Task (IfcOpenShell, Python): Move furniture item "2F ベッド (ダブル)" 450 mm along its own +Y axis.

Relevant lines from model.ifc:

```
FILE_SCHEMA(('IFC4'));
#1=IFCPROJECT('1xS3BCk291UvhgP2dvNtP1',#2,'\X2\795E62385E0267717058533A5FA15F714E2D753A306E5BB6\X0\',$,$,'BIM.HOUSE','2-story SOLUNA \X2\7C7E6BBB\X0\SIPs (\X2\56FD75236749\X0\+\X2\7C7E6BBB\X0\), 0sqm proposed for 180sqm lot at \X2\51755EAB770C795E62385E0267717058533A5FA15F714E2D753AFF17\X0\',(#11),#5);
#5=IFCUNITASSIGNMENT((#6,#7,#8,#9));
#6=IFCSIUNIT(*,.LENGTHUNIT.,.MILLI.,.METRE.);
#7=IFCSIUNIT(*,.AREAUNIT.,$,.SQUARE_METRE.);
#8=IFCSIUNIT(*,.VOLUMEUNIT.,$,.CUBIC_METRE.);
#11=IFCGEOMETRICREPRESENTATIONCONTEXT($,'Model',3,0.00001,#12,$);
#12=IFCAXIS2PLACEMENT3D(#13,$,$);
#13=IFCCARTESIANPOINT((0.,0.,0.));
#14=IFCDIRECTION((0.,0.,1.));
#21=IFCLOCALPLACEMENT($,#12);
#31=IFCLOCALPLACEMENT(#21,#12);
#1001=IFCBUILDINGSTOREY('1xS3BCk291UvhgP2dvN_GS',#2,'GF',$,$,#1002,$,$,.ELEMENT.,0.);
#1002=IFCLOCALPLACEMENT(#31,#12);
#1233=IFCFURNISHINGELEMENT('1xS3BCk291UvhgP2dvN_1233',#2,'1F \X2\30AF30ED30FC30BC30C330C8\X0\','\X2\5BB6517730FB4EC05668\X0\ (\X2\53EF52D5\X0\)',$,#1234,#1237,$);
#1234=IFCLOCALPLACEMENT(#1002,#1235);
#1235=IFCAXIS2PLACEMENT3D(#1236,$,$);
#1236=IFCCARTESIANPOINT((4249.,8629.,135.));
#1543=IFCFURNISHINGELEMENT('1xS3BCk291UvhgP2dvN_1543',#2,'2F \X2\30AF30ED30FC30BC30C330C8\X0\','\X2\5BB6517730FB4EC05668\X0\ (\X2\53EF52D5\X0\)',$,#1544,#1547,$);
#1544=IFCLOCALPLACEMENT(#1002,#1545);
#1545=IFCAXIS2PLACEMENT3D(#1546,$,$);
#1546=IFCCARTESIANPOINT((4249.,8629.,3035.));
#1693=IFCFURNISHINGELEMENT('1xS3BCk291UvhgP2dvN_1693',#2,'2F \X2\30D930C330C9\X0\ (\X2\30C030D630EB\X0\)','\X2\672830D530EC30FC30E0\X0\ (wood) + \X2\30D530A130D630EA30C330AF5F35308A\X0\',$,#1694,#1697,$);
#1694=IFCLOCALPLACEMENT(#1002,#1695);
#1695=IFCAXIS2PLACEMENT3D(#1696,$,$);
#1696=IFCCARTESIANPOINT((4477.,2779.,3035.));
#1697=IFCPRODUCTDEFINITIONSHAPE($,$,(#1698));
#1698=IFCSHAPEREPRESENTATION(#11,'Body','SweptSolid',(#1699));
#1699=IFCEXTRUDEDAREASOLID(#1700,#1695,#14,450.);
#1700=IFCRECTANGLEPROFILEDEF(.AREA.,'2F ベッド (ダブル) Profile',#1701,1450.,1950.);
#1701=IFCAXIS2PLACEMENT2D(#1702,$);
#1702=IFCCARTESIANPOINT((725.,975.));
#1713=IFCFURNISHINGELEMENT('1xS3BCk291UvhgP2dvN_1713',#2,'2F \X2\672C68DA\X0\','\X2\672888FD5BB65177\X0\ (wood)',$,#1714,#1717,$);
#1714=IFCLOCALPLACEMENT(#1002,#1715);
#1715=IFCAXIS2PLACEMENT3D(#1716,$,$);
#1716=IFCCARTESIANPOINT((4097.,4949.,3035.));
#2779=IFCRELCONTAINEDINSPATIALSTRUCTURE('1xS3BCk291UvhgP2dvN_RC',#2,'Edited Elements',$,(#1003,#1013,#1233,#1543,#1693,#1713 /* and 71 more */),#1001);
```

```python
import ifcopenshell
import ifcopenshell.api.geometry
import ifcopenshell.util.placement

model = ifcopenshell.open("model.ifc")

item = model.by_guid("1xS3BCk291UvhgP2dvN_1693")
matrix = ifcopenshell.util.placement.get_local_placement(item.ObjectPlacement)
matrix[:3, 3] += matrix[:3, 1] * 450.0
ifcopenshell.api.geometry.edit_object_placement(model, product=item, matrix=matrix, is_si=False)

print(ifcopenshell.util.placement.get_local_placement(item.ObjectPlacement).round(3) + 0.0)

model.write("model_rev.ifc")
```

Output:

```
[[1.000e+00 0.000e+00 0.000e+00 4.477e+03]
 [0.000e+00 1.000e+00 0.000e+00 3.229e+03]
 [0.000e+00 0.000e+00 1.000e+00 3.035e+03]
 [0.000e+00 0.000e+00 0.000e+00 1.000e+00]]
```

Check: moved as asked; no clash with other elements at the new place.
